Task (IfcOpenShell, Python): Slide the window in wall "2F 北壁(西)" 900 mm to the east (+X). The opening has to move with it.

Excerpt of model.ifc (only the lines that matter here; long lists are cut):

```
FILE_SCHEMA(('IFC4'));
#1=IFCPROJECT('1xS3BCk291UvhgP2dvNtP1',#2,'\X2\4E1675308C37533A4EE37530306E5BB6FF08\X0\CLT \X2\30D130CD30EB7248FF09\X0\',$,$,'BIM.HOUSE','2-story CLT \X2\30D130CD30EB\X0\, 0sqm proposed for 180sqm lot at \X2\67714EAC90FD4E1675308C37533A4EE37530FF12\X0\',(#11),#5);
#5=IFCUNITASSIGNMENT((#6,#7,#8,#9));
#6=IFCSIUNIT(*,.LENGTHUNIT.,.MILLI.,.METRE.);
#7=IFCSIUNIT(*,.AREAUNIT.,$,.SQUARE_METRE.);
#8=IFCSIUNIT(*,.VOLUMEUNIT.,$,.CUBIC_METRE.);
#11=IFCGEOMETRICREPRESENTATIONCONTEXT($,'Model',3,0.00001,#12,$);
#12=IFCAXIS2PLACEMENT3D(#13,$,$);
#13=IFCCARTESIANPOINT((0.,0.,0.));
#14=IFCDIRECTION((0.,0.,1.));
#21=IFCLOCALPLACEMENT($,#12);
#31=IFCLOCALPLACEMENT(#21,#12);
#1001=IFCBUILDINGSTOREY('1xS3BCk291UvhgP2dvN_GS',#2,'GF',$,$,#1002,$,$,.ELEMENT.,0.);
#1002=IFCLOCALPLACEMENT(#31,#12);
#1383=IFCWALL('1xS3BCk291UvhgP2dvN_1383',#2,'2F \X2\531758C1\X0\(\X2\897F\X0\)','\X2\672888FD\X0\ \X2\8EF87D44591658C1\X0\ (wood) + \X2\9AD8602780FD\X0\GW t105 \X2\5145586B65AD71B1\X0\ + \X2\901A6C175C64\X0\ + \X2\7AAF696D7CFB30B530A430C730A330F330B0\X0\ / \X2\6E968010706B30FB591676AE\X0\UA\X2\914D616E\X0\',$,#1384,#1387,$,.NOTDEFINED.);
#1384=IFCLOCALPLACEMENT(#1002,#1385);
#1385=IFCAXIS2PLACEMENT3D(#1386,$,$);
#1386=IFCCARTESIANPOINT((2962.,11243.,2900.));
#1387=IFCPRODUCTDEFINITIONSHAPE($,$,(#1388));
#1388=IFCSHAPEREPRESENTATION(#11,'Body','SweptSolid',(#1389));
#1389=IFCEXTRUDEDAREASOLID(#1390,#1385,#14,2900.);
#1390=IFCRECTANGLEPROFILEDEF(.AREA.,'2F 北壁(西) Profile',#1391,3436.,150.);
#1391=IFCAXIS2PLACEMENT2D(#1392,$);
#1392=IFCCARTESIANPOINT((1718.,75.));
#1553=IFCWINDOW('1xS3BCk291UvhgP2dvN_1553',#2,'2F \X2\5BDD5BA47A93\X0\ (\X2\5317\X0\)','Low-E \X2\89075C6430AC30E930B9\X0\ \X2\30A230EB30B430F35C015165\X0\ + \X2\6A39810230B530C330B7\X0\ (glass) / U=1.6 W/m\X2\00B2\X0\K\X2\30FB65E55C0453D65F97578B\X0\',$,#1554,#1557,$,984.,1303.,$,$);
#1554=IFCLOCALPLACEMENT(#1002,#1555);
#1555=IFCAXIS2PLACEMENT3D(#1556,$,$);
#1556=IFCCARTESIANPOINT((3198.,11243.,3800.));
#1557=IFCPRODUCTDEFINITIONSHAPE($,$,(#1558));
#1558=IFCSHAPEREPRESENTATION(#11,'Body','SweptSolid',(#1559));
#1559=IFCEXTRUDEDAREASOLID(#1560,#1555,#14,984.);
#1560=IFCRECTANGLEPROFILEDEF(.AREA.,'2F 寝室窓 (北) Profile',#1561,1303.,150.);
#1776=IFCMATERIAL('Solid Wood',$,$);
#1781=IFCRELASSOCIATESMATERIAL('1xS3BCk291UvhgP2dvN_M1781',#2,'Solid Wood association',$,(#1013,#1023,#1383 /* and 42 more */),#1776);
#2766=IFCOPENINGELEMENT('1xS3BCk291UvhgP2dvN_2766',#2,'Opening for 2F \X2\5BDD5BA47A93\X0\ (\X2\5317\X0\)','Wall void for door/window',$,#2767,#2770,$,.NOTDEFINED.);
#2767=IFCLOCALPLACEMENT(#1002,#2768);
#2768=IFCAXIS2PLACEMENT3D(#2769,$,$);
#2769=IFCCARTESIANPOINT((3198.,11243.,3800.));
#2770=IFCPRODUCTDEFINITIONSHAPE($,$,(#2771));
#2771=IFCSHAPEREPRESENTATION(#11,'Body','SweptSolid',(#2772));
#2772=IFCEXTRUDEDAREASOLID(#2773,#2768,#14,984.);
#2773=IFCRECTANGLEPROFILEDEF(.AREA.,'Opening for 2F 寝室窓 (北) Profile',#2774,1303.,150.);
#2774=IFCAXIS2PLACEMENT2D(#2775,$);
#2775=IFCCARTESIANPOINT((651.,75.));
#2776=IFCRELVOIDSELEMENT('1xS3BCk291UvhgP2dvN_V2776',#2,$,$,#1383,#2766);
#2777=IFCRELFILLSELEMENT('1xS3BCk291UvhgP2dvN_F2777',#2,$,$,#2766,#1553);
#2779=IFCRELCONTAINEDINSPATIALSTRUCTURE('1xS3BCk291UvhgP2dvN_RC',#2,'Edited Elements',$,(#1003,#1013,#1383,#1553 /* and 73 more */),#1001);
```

```python
import ifcopenshell
import ifcopenshell.api.geometry
import ifcopenshell.util.placement

model = ifcopenshell.open("model.ifc")

window = model.by_guid("1xS3BCk291UvhgP2dvN_1553")
opening = window.FillsVoids[0].RelatingOpeningElement
wall = opening.VoidsElements[0].RelatingBuildingElement

wall_matrix = ifcopenshell.util.placement.get_local_placement(wall.ObjectPlacement)
shift = wall_matrix[:3, 0] * 900.0
before = ifcopenshell.util.placement.get_local_placement(window.ObjectPlacement)[:3, 3].copy()

# The window is not placed relative to its opening, so move both.
for product in (opening, window):
    matrix = ifcopenshell.util.placement.get_local_placement(product.ObjectPlacement)
    matrix[:3, 3] += shift
    ifcopenshell.api.geometry.edit_object_placement(model, product=product, matrix=matrix, is_si=False)

after = ifcopenshell.util.placement.get_local_placement(window.ObjectPlacement)[:3, 3]
print("window moved by", (after - before).round(3) + 0.0)

model.write("model_rev.ifc")
```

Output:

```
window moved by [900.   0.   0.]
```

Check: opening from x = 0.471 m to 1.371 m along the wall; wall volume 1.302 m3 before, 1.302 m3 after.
